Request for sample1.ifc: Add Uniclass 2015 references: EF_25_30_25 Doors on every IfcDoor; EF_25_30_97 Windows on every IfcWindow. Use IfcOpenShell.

First a look at what the model holds.

```python
import ifcopenshell

model = ifcopenshell.open("sample1.ifc")
print(model.schema)
print("classifications:", [c.Name for c in model.by_type("IfcClassification")])
for ifc_class in ("IfcDoor", "IfcRoof", "IfcStair", "IfcWall", "IfcWindow"):
    print(ifc_class, len(model.by_type(ifc_class)))
```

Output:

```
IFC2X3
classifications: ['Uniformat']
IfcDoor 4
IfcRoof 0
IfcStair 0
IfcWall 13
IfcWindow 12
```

```python
import ifcopenshell
import ifcopenshell.api.classification

model = ifcopenshell.open("sample1.ifc")

# IFC2X3 requires Source and Edition and has no link from the project to the system.
system = model.create_entity("IfcClassification", Source="NBS", Edition="2015", Name="Uniclass 2015")

codes = {
    "IfcDoor": ("EF_25_30_25", "Doors"),
    "IfcWindow": ("EF_25_30_97", "Windows"),
}
for ifc_class, (code, name) in codes.items():
    products = model.by_type(ifc_class)
    ifcopenshell.api.classification.add_reference(
        model, products=products, classification=system, identification=code, name=name
    )
    print(code, len(products))

model.write("sample1_v2.ifc")
```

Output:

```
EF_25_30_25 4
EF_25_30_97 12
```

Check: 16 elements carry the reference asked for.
